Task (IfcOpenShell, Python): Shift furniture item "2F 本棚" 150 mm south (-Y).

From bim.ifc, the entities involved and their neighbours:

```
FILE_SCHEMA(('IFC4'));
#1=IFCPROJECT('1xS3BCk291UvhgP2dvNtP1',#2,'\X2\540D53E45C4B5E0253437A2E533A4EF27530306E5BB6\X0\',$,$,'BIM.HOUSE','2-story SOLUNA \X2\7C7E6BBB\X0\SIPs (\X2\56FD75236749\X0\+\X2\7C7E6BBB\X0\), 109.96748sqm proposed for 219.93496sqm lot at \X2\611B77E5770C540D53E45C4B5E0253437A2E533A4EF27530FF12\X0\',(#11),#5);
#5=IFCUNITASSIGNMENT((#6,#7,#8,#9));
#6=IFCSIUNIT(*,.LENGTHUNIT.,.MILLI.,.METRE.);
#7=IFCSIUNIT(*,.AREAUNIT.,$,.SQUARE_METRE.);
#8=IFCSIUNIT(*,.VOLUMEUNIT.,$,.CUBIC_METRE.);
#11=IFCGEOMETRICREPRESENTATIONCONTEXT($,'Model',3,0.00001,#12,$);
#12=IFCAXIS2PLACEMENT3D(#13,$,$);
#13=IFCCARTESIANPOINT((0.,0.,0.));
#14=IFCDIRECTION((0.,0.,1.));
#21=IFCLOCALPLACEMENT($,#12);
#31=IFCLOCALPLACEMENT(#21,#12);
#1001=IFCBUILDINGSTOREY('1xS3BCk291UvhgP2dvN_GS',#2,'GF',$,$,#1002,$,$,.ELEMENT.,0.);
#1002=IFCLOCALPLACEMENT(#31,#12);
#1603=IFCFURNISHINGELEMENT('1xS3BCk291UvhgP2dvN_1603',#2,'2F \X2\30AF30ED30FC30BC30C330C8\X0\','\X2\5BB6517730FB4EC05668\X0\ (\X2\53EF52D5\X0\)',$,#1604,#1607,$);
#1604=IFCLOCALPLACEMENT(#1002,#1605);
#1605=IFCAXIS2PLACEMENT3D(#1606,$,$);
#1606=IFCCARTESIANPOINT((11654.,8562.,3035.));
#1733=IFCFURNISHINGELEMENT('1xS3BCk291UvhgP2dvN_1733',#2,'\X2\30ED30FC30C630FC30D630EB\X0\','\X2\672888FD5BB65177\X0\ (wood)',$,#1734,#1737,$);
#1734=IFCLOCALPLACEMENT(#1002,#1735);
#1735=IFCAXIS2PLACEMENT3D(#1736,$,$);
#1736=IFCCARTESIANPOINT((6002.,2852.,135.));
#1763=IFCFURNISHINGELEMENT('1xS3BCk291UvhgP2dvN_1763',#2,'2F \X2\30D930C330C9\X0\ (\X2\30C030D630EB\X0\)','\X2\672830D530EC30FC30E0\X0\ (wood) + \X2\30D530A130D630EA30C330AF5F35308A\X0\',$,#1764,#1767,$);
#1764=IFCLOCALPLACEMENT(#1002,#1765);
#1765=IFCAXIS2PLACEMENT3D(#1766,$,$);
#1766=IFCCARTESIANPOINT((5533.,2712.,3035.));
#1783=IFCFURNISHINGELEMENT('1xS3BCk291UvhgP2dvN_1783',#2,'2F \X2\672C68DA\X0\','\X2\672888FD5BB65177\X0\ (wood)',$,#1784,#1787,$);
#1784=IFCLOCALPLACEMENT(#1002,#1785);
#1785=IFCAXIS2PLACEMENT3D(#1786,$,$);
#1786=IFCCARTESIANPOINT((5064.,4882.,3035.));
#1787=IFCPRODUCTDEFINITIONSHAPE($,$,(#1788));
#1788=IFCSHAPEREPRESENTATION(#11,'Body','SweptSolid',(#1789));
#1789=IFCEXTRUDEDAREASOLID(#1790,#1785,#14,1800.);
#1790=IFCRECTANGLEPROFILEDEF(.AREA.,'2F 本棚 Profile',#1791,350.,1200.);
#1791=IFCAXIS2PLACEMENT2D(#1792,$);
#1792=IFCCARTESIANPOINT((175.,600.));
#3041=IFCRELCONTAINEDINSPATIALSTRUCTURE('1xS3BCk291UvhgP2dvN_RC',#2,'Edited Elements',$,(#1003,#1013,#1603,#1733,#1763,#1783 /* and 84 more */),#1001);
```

```python
import ifcopenshell
import ifcopenshell.api.geometry
import ifcopenshell.util.placement

model = ifcopenshell.open("bim.ifc")

item = model.by_guid("1xS3BCk291UvhgP2dvN_1783")
matrix = ifcopenshell.util.placement.get_local_placement(item.ObjectPlacement)
matrix[1, 3] -= 150.0
ifcopenshell.api.geometry.edit_object_placement(model, product=item, matrix=matrix, is_si=False)

print(ifcopenshell.util.placement.get_local_placement(item.ObjectPlacement).round(3) + 0.0)

model.write("bim_updated.ifc")
```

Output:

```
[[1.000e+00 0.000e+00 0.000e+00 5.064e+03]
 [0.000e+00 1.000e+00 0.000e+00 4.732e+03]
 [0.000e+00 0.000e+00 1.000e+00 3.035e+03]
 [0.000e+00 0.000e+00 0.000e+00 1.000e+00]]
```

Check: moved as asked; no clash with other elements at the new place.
